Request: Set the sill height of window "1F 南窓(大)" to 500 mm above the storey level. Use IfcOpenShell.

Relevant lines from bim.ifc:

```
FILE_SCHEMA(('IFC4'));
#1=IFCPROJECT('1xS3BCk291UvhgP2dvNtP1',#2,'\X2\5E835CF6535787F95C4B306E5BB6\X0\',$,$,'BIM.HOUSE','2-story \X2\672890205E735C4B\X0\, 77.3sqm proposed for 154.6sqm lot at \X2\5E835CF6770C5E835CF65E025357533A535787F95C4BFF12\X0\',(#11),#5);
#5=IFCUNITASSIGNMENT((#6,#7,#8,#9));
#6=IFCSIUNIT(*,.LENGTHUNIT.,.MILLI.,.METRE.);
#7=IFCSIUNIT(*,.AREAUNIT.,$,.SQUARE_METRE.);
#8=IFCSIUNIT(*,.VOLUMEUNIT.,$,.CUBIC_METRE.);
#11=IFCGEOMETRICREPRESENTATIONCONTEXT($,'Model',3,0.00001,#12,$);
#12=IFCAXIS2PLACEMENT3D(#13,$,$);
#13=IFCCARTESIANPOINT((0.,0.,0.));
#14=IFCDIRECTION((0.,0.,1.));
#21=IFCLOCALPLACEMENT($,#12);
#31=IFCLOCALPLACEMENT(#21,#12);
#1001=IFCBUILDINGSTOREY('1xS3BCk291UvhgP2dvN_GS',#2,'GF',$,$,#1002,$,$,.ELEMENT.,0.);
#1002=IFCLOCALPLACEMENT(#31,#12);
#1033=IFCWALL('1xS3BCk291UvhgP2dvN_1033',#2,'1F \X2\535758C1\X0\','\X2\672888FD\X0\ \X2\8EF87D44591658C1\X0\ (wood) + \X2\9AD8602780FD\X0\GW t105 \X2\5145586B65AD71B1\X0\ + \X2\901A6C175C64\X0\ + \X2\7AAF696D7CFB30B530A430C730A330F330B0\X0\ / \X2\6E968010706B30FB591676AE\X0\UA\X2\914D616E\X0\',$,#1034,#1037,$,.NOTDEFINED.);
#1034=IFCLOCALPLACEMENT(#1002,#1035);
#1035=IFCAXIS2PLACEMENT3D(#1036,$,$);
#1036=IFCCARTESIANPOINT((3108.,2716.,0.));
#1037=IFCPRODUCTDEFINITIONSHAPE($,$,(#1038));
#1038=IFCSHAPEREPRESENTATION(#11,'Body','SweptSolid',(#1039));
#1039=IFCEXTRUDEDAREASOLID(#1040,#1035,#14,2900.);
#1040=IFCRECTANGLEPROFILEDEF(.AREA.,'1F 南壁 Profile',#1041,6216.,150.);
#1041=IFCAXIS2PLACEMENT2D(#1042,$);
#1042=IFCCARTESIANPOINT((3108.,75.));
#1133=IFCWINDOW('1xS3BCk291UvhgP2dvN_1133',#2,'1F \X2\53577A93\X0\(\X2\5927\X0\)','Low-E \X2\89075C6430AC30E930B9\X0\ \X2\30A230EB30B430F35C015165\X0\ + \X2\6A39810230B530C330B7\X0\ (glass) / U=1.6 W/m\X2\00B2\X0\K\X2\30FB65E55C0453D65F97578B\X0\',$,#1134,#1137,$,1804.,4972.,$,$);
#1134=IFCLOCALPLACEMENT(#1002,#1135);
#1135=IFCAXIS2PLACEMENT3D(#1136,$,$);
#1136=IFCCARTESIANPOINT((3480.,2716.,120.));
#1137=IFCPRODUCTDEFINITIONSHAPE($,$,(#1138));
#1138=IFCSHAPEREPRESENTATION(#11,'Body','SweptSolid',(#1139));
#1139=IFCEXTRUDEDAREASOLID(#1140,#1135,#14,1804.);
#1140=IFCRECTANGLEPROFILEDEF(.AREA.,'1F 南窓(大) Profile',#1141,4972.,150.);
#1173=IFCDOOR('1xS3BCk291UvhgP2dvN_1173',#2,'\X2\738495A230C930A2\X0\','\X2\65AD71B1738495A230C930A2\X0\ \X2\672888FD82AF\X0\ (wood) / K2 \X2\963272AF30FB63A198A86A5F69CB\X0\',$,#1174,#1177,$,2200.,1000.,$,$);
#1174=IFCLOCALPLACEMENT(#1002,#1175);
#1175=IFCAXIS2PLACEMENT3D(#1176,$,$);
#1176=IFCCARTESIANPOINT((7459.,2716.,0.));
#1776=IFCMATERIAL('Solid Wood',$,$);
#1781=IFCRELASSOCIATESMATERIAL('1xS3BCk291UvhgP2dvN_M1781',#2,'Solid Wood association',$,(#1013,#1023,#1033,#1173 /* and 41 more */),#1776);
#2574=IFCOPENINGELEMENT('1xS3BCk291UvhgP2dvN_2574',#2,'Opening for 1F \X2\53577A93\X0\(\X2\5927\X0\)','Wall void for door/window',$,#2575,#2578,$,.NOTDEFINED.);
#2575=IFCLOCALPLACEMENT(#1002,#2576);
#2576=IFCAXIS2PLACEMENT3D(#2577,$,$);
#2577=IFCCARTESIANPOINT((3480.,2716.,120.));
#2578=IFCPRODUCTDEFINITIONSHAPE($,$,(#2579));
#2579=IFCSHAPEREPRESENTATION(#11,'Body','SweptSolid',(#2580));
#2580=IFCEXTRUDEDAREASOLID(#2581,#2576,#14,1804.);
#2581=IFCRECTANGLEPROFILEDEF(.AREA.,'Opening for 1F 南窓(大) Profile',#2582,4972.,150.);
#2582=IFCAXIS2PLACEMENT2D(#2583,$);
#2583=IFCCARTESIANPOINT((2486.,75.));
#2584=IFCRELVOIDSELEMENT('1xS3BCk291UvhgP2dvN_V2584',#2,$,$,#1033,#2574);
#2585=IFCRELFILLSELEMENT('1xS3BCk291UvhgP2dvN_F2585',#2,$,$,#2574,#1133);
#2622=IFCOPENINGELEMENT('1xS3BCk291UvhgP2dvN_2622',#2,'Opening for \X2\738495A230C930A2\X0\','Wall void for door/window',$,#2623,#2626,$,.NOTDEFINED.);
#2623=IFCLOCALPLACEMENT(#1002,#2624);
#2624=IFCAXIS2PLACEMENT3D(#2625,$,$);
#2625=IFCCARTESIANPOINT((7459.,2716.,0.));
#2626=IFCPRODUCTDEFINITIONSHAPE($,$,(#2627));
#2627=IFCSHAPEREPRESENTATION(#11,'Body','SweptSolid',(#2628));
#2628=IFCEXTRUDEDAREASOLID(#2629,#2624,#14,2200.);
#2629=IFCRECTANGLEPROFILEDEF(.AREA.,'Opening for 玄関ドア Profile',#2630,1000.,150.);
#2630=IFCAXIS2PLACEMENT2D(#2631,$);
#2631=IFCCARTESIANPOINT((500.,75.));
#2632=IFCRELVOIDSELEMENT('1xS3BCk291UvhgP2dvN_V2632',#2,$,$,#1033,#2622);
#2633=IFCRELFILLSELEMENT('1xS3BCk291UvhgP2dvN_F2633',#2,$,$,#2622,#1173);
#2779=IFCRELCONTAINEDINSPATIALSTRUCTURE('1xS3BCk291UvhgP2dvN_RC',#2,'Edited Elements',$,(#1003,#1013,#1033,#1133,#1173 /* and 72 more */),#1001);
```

```python
import numpy as np
import ifcopenshell
import ifcopenshell.api.geometry
import ifcopenshell.geom
import ifcopenshell.util.element
import ifcopenshell.util.placement
import ifcopenshell.util.shape
import ifcopenshell.util.unit

model = ifcopenshell.open("bim.ifc")
unit_scale = ifcopenshell.util.unit.calculate_unit_scale(model)

window = model.by_guid("1xS3BCk291UvhgP2dvN_1133")
opening = window.FillsVoids[0].RelatingOpeningElement
storey = ifcopenshell.util.element.get_container(window, ifc_class="IfcBuildingStorey")
level = ifcopenshell.util.placement.get_local_placement(storey.ObjectPlacement)[2, 3]

# The opening's origin need not be at the sill, so measure its lowest point.
shape = ifcopenshell.geom.create_shape(ifcopenshell.geom.settings(), opening)
bottom = ifcopenshell.util.shape.get_shape_bottom_elevation(shape, shape.geometry) / unit_scale
dz = level + 0.5 / unit_scale - bottom

shift = np.array([0.0, 0.0, dz])
# The window is not placed relative to its opening, so move both.
for product in (opening, window):
    matrix = ifcopenshell.util.placement.get_local_placement(product.ObjectPlacement)
    matrix[:3, 3] += shift
    ifcopenshell.api.geometry.edit_object_placement(model, product=product, matrix=matrix, is_si=False)

print(f"moved by {dz * unit_scale:+.3f} m")

model.write("bim_updated.ifc")
```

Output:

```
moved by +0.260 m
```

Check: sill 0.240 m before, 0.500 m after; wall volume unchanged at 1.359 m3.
